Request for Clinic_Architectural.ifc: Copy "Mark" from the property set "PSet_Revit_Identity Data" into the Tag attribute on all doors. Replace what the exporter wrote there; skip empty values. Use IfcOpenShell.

First a look at what the model holds.

```python
import ifcopenshell
import ifcopenshell.util.element

model = ifcopenshell.open("Clinic_Architectural.ifc")
print(model.schema)
doors = model.by_type("IfcDoor")
print(len(doors), "doors")
for e in doors[:8]:
    source = ifcopenshell.util.element.get_pset(e, "PSet_Revit_Identity Data", "Mark")
    target = e.Tag
    print(e.id(), repr(source), repr(target), sep=" | ")
```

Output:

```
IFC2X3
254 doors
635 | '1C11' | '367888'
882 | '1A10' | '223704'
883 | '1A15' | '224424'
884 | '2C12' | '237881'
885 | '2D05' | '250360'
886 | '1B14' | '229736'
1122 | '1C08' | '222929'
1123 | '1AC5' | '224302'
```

```python
import ifcopenshell
import ifcopenshell.util.element

model = ifcopenshell.open("Clinic_Architectural.ifc")

count = 0
for e in model.by_type("IfcDoor"):
    value = ifcopenshell.util.element.get_pset(e, "PSet_Revit_Identity Data", "Mark")
    current = e.Tag
    if not value or not value.strip() or current == value:
        continue
    e.Tag = value
    count += 1

print(count, "doors updated")

model.write("Clinic_Architectural-out.ifc")
```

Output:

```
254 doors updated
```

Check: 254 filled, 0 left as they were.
